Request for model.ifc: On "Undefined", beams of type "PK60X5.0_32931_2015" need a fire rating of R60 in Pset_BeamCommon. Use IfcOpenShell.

First a look at what the model holds.

```python
import ifcopenshell
import ifcopenshell.util.element

model = ifcopenshell.open("model.ifc")
print(model.schema)
storey = next(s for s in model.by_type("IfcBuildingStorey") if s.Name == "Undefined")
beams = [e for e in ifcopenshell.util.element.get_decomposition(storey) if e.is_a("IfcBeam")]
seen = {}
for e in beams:
    element_type = ifcopenshell.util.element.get_type(e)
    key = (element_type.Name if element_type != e and element_type else None, ifcopenshell.util.element.get_pset(e, "Pset_BeamCommon", "FireRating"))
    seen[key] = seen.get(key, 0) + 1
for (name, value), count in sorted(seen.items(), key=str):
    print(count, "x", name, "|", value)
```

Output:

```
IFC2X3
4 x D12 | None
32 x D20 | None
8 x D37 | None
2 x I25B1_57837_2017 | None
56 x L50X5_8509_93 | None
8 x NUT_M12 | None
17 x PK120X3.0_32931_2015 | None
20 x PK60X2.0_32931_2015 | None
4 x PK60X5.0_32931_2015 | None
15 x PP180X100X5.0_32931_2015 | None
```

```python
import ifcopenshell
import ifcopenshell.api.pset
import ifcopenshell.util.element

model = ifcopenshell.open("model.ifc")

storey = next(s for s in model.by_type("IfcBuildingStorey") if s.Name == "Undefined")
beams = [e for e in ifcopenshell.util.element.get_decomposition(storey) if e.is_a("IfcBeam")]

count = 0
for e in beams:
    element_type = ifcopenshell.util.element.get_type(e)
    if element_type in (None, e) or element_type.Name != "PK60X5.0_32931_2015":
        continue
    found = ifcopenshell.util.element.get_pset(e, "Pset_BeamCommon", should_inherit=False)
    if found:
        pset = model.by_id(found["id"])
        if len(ifcopenshell.util.element.get_elements_by_pset(pset)) > 1:
            pset = ifcopenshell.api.pset.unshare_pset(model, products=[e], pset=pset)[0]
    else:
        pset = ifcopenshell.api.pset.add_pset(model, product=e, name="Pset_BeamCommon")
    ifcopenshell.api.pset.edit_pset(model, pset=pset, properties={"FireRating": "R60"})
    count += 1

print(count, "beams updated")

model.write("model_edited.ifc")
```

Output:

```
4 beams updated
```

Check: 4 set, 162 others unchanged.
